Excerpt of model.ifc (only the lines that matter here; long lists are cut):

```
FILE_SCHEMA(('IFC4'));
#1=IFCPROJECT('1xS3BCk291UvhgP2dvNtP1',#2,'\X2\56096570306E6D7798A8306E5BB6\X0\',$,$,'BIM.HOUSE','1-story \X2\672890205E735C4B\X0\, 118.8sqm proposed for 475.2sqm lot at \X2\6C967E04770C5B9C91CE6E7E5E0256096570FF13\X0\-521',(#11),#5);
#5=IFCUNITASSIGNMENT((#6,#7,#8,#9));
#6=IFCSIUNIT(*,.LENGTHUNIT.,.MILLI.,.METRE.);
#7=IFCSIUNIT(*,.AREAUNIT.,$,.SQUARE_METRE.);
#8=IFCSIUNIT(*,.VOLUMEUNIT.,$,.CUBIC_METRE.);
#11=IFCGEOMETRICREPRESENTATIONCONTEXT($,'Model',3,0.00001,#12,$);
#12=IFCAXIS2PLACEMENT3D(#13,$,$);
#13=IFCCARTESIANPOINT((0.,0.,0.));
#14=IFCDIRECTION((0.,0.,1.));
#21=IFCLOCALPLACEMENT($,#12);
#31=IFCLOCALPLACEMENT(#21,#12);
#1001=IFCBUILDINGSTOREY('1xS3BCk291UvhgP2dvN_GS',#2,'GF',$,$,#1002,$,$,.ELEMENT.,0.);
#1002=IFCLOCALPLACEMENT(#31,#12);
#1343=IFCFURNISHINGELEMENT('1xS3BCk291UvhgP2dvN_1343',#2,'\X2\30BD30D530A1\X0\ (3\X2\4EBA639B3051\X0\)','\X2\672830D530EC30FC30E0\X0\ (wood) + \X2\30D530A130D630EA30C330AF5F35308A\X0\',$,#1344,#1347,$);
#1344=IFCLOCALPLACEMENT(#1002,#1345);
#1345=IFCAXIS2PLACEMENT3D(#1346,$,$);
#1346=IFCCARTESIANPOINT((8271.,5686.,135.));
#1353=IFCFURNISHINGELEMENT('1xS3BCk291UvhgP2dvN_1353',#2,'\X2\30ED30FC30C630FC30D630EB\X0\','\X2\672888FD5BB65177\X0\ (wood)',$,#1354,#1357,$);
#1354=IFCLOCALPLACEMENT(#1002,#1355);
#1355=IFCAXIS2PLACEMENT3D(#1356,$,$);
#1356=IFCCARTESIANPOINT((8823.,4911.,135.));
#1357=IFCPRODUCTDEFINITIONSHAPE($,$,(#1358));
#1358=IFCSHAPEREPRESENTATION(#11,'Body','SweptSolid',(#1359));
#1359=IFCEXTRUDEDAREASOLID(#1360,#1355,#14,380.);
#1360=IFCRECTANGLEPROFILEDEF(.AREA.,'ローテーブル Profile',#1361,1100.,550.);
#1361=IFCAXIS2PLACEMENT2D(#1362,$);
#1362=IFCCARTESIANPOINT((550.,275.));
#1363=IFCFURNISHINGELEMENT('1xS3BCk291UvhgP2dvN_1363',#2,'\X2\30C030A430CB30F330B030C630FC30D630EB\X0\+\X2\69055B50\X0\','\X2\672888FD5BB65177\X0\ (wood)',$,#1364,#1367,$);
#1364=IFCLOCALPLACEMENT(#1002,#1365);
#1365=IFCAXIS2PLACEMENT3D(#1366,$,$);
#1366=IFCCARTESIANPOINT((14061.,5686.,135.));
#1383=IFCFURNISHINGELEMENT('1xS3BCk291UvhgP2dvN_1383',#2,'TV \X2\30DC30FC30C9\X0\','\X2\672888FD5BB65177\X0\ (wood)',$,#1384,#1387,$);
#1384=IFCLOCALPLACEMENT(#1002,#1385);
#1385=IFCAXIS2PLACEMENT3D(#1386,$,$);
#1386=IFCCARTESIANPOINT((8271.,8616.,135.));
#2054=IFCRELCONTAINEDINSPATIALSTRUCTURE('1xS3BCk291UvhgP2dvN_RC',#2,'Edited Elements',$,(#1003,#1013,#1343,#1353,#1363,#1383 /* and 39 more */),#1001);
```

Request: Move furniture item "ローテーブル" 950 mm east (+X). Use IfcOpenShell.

```python
import ifcopenshell
import ifcopenshell.api.geometry
import ifcopenshell.util.placement
import ifcopenshell.util.unit

model = ifcopenshell.open("model.ifc")
unit_scale = ifcopenshell.util.unit.calculate_unit_scale(model)

item = model.by_guid("1xS3BCk291UvhgP2dvN_1353")
matrix = ifcopenshell.util.placement.get_local_placement(item.ObjectPlacement)
matrix[0, 3] += 0.95 / unit_scale
ifcopenshell.api.geometry.edit_object_placement(model, product=item, matrix=matrix, is_si=False)

print(ifcopenshell.util.placement.get_local_placement(item.ObjectPlacement).round(3) + 0.0)

model.write("model-out.ifc")
```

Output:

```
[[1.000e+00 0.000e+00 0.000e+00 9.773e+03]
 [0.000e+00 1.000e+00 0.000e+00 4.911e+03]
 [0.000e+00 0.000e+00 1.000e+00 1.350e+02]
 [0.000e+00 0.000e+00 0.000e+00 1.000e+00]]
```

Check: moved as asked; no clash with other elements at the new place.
